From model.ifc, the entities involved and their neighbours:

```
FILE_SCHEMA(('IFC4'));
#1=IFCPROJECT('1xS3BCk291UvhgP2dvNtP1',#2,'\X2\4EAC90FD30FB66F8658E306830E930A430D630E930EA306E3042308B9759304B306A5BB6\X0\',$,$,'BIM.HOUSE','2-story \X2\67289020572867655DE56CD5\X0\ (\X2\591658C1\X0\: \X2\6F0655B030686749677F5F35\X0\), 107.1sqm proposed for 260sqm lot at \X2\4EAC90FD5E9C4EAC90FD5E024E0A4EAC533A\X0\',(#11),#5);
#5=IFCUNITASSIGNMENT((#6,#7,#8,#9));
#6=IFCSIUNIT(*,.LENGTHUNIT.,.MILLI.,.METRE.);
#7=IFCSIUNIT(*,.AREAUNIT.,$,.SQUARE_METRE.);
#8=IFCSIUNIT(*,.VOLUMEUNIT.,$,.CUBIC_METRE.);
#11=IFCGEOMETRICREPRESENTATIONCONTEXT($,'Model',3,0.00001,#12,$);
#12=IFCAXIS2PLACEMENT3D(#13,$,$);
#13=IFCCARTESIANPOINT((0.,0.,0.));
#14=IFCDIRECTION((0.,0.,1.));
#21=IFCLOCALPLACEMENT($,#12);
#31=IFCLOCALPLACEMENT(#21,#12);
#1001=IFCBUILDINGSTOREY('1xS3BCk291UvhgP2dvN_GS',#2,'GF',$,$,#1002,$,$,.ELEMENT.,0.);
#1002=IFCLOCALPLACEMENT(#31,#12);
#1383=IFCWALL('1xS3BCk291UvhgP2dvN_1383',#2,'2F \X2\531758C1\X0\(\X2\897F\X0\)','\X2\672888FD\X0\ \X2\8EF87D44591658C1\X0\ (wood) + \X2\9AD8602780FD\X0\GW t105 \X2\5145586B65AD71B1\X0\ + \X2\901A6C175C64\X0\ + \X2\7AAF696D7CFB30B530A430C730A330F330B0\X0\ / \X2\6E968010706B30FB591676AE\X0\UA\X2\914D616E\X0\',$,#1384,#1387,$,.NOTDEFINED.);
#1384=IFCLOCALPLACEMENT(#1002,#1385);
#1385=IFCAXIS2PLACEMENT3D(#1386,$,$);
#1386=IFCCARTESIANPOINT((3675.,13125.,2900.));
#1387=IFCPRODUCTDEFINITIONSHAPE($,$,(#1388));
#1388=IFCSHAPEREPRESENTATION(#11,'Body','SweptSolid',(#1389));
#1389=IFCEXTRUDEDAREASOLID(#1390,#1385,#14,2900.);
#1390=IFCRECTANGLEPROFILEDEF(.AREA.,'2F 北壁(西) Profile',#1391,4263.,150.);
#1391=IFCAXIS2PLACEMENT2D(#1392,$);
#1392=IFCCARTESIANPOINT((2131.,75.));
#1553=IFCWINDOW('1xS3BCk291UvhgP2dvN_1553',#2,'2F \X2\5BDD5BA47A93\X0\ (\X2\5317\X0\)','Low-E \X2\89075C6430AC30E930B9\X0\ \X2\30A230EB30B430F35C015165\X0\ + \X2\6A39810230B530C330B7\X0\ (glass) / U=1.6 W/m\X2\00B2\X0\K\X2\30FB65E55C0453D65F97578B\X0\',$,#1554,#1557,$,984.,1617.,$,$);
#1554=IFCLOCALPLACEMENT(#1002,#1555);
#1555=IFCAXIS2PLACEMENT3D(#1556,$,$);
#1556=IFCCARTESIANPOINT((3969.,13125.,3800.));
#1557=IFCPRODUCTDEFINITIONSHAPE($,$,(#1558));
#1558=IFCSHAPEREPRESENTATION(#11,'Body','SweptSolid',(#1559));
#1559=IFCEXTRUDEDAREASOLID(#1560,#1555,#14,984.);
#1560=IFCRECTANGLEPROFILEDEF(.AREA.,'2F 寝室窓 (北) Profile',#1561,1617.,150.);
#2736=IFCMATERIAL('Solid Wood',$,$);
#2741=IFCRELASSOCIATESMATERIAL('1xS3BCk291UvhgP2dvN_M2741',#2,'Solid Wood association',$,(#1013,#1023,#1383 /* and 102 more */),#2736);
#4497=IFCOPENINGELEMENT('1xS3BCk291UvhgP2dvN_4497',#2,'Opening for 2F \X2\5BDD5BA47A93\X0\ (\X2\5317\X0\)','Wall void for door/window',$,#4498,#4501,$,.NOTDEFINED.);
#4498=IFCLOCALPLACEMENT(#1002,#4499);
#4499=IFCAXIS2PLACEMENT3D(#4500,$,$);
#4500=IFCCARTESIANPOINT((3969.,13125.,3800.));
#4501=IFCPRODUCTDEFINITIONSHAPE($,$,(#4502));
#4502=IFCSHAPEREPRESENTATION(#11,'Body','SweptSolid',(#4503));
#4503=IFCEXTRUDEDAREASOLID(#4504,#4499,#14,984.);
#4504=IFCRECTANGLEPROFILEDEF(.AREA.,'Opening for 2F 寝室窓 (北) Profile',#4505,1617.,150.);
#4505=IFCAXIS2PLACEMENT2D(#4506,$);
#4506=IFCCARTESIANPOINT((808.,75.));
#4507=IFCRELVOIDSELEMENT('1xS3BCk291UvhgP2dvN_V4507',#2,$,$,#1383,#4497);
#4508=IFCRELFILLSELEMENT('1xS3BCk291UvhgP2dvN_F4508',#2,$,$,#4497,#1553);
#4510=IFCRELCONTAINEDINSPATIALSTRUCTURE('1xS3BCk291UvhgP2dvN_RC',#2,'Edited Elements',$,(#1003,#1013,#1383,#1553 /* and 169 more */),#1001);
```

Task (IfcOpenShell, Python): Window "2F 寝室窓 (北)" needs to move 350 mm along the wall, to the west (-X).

```python
import ifcopenshell
import ifcopenshell.api.geometry
import ifcopenshell.util.placement
import ifcopenshell.util.unit

model = ifcopenshell.open("model.ifc")
unit_scale = ifcopenshell.util.unit.calculate_unit_scale(model)

window = model.by_guid("1xS3BCk291UvhgP2dvN_1553")
opening = window.FillsVoids[0].RelatingOpeningElement
wall = opening.VoidsElements[0].RelatingBuildingElement

wall_matrix = ifcopenshell.util.placement.get_local_placement(wall.ObjectPlacement)
shift = wall_matrix[:3, 0] * -0.35 / unit_scale
before = ifcopenshell.util.placement.get_local_placement(window.ObjectPlacement)[:3, 3].copy()

# The window is not placed relative to its opening, so move both.
for product in (opening, window):
    matrix = ifcopenshell.util.placement.get_local_placement(product.ObjectPlacement)
    matrix[:3, 3] += shift
    ifcopenshell.api.geometry.edit_object_placement(model, product=product, matrix=matrix, is_si=False)

after = ifcopenshell.util.placement.get_local_placement(window.ObjectPlacement)[:3, 3]
print("window moved by", (after - before).round(3) + 0.0)

model.write("model_rev.ifc")
```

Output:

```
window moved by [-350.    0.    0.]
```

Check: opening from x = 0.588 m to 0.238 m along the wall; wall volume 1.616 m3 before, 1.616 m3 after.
